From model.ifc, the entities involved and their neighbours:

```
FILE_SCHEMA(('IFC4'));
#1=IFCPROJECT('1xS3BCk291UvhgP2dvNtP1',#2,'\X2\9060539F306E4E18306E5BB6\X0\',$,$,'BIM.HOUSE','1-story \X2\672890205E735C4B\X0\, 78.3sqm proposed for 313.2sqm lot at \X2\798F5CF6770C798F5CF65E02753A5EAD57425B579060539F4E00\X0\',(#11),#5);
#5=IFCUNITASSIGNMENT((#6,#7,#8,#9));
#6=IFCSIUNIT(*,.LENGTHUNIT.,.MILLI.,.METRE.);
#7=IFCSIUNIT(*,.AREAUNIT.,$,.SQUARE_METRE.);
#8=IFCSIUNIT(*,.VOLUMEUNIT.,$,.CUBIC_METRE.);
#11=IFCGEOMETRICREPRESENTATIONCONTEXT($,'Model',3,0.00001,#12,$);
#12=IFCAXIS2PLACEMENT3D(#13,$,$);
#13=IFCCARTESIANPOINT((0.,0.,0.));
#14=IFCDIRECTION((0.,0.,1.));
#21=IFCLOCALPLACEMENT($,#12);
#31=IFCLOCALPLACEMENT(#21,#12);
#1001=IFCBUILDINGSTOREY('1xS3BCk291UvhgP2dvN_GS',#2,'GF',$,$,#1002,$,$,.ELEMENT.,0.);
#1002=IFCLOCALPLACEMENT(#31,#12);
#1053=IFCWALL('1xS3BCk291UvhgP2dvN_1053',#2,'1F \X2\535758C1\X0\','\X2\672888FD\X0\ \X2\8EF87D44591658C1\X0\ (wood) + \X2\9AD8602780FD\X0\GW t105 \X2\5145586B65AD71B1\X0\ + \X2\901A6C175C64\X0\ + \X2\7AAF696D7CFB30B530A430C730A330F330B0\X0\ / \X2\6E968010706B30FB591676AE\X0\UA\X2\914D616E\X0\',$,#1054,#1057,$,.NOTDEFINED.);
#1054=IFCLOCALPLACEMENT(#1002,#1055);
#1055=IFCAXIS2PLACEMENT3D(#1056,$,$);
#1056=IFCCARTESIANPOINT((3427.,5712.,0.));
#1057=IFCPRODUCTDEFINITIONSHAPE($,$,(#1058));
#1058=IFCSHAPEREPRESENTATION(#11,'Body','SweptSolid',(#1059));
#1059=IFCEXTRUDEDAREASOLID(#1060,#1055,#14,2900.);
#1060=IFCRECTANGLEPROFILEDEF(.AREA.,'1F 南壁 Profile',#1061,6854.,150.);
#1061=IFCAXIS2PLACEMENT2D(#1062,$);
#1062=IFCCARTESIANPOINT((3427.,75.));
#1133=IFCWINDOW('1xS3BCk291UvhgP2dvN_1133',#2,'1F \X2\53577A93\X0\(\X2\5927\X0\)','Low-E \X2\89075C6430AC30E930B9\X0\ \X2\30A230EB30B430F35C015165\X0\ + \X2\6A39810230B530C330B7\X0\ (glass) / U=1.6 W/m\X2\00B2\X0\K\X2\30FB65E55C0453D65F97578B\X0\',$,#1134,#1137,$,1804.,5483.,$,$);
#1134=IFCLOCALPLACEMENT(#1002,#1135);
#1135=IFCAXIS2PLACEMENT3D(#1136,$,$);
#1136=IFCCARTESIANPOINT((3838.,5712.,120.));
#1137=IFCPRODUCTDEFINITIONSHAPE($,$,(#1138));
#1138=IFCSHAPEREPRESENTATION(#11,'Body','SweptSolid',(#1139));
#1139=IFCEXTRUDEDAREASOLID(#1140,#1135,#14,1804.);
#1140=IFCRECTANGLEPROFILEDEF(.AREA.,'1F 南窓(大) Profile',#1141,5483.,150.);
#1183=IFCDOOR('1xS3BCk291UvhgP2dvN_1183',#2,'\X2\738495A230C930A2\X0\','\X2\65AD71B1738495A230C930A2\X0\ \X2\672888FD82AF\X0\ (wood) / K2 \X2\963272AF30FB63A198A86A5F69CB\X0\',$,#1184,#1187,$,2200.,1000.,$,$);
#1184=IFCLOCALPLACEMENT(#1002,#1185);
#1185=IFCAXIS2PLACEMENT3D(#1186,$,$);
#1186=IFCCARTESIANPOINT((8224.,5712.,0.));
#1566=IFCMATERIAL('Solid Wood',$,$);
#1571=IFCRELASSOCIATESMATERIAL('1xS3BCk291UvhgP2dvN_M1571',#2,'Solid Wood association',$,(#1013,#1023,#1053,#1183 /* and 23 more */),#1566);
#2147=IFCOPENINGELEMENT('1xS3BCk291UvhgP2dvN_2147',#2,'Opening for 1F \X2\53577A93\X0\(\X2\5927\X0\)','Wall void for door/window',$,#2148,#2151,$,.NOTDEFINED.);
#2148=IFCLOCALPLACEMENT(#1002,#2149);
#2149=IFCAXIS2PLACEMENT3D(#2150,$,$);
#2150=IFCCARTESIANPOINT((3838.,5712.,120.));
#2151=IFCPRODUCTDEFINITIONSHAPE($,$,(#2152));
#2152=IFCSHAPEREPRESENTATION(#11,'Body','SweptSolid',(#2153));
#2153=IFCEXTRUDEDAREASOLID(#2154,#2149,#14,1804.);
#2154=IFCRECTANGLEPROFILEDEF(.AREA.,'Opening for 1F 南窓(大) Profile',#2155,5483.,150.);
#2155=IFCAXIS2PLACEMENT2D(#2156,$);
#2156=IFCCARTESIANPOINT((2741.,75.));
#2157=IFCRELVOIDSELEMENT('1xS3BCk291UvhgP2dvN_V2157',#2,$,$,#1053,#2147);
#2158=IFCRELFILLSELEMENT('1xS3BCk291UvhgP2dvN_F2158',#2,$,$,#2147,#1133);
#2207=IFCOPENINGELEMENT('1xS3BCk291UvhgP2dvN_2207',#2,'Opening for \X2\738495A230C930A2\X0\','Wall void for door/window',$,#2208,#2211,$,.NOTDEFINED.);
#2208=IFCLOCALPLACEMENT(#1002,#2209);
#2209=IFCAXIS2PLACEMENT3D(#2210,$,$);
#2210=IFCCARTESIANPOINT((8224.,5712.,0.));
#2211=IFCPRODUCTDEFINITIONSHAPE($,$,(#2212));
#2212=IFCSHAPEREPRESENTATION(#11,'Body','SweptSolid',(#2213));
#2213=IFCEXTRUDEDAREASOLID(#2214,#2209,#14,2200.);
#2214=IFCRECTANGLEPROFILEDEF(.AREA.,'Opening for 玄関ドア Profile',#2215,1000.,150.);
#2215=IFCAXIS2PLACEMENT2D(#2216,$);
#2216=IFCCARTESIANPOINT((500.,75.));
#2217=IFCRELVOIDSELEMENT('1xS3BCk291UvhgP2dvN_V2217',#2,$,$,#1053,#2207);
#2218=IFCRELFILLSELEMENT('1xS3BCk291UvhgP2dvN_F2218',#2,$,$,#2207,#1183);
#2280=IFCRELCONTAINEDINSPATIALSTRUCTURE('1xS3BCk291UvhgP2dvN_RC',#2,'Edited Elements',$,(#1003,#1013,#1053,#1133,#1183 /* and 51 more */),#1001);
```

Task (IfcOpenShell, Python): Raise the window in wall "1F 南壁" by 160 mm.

```python
import numpy as np
import ifcopenshell
import ifcopenshell.api.geometry
import ifcopenshell.util.placement
import ifcopenshell.util.unit

model = ifcopenshell.open("model.ifc")
unit_scale = ifcopenshell.util.unit.calculate_unit_scale(model)

window = model.by_guid("1xS3BCk291UvhgP2dvN_1133")
opening = window.FillsVoids[0].RelatingOpeningElement
dz = 0.16 / unit_scale

shift = np.array([0.0, 0.0, dz])
# The window is not placed relative to its opening, so move both.
for product in (opening, window):
    matrix = ifcopenshell.util.placement.get_local_placement(product.ObjectPlacement)
    matrix[:3, 3] += shift
    ifcopenshell.api.geometry.edit_object_placement(model, product=product, matrix=matrix, is_si=False)

print(f"moved by {dz * unit_scale:+.3f} m")

model.write("model-out.ifc")
```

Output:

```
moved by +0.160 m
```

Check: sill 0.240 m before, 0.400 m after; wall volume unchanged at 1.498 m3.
